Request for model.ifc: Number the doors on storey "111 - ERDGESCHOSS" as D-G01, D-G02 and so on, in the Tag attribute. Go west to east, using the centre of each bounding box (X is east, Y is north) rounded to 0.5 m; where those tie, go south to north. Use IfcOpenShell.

First a look at what the model holds.

```python
import ifcopenshell
import ifcopenshell.util.element
import ifcopenshell.util.placement

model = ifcopenshell.open("model.ifc")
print(model.schema)
storey = next(s for s in model.by_type("IfcBuildingStorey") if s.Name == "111 - ERDGESCHOSS")
doors = [e for e in ifcopenshell.util.element.get_decomposition(storey) if e.is_a("IfcDoor")]
for e in sorted(doors, key=lambda e: e.id()):
    origin = ifcopenshell.util.placement.get_local_placement(e.ObjectPlacement)[:3, 3]
    print(e.id(), e.Tag, e.Name, origin.round(2) + 0.0, sep=" | ")
```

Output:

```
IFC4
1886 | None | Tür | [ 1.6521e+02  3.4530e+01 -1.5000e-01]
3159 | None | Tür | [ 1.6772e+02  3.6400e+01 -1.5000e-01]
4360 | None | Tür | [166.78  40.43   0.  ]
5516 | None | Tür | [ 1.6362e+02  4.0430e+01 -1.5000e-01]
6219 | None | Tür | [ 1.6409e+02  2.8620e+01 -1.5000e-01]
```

```python
import ifcopenshell
import ifcopenshell.geom
import ifcopenshell.util.element
import ifcopenshell.util.shape

model = ifcopenshell.open("model.ifc")
settings = ifcopenshell.geom.settings()
settings.set("use-world-coords", True)


def centre(element):
    shape = ifcopenshell.geom.create_shape(settings, element)
    return ifcopenshell.util.shape.get_bbox_centroid(shape.geometry)


storey = next(s for s in model.by_type("IfcBuildingStorey") if s.Name == "111 - ERDGESCHOSS")
doors = [e for e in ifcopenshell.util.element.get_decomposition(storey) if e.is_a("IfcDoor")]

# Insertion points can sit at a corner or the storey origin, so sort by the geometry (in metres).
centres = {e: centre(e) for e in doors}
doors.sort(key=lambda e: (round(centres[e][0] / 0.5), centres[e][1]))

for i, e in enumerate(doors, start=1):
    number = f"D-G{i:02d}"
    e.Tag = number
    print(e.id(), number)

model.write("model_v2.ifc")
```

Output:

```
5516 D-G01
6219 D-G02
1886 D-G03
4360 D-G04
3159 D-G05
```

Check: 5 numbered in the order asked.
